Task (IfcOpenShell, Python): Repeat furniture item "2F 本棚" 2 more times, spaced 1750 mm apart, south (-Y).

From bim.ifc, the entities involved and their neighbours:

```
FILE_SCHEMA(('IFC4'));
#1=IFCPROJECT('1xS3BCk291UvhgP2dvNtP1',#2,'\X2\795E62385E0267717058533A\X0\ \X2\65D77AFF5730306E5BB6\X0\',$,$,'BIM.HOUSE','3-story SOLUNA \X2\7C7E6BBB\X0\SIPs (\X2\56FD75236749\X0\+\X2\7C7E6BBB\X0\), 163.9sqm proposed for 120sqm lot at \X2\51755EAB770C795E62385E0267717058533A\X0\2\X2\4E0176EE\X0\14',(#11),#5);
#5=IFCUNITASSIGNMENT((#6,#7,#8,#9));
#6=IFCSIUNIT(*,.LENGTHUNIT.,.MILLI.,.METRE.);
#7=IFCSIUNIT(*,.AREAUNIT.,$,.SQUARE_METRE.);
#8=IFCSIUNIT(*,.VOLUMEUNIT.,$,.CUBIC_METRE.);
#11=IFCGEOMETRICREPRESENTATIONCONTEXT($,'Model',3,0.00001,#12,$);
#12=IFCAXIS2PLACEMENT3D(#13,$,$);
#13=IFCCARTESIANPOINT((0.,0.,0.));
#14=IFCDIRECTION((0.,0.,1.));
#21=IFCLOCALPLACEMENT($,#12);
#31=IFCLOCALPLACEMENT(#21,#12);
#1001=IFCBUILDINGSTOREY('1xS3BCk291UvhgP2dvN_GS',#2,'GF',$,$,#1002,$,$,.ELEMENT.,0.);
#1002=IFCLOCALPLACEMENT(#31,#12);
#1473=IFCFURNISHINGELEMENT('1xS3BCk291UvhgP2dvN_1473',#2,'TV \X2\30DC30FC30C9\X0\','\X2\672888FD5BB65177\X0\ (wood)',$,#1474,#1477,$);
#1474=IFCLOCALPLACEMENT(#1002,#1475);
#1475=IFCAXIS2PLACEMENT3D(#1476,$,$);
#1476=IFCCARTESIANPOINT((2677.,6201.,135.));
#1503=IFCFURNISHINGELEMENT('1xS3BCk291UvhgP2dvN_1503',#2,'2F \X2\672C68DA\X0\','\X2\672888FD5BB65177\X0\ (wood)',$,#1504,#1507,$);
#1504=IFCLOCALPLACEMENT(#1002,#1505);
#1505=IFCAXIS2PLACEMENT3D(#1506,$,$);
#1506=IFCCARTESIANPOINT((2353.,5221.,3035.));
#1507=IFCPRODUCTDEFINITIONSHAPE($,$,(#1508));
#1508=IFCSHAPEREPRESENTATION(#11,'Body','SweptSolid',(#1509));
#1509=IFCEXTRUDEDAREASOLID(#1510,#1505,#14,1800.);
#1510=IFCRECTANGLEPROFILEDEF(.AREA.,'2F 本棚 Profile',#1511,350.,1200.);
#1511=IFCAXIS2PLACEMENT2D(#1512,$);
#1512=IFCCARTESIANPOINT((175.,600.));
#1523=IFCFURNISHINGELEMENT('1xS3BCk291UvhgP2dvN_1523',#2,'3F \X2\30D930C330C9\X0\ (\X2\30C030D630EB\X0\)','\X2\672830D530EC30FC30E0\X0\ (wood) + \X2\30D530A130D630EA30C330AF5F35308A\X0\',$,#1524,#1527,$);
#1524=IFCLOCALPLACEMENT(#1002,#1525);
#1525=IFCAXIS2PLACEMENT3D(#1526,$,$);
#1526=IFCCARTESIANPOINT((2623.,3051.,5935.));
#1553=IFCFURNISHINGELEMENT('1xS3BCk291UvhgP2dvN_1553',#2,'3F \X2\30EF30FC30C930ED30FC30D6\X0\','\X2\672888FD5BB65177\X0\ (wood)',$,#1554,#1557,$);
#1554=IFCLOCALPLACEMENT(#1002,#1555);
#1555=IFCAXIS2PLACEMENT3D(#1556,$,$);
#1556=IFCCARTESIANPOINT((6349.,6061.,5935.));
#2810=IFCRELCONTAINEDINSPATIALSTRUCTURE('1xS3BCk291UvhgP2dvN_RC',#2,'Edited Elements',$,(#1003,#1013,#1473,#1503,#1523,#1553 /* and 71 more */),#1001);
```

```python
import numpy as np
import ifcopenshell
import ifcopenshell.api.geometry
import ifcopenshell.api.root
import ifcopenshell.util.element
import ifcopenshell.util.placement

model = ifcopenshell.open("bim.ifc")


def reuse_history(source, copy):
    """copy_class also copies each property set's owner history, people and application; keep the originals."""
    for rel in copy.IsDefinedBy:
        if rel.is_a("IfcRelDefinesByProperties") and (history := rel.RelatingPropertyDefinition.OwnerHistory):
            rel.RelatingPropertyDefinition.OwnerHistory = source.OwnerHistory
            ifcopenshell.util.element.remove_deep2(model, history)


source = model.by_id(1503)
base = ifcopenshell.util.placement.get_local_placement(source.ObjectPlacement)
step = np.array([0.0, -1.0, 0.0]) * 1750.0

for i in range(1, 3):
    copy = ifcopenshell.api.root.copy_class(model, product=source)
    copy.Representation = ifcopenshell.util.element.copy_deep(
        model, source.Representation, exclude=["IfcGeometricRepresentationContext", "IfcRepresentationMap"]
    )
    reuse_history(source, copy)
    matrix = base.copy()
    matrix[:3, 3] += i * step
    print("added at", matrix[:3, 3].round(3) + 0.0)
    ifcopenshell.api.geometry.edit_object_placement(model, product=copy, matrix=matrix, is_si=False)

model.write("bim-out.ifc")
```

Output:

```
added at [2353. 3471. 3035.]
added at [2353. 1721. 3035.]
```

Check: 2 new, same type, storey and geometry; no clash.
